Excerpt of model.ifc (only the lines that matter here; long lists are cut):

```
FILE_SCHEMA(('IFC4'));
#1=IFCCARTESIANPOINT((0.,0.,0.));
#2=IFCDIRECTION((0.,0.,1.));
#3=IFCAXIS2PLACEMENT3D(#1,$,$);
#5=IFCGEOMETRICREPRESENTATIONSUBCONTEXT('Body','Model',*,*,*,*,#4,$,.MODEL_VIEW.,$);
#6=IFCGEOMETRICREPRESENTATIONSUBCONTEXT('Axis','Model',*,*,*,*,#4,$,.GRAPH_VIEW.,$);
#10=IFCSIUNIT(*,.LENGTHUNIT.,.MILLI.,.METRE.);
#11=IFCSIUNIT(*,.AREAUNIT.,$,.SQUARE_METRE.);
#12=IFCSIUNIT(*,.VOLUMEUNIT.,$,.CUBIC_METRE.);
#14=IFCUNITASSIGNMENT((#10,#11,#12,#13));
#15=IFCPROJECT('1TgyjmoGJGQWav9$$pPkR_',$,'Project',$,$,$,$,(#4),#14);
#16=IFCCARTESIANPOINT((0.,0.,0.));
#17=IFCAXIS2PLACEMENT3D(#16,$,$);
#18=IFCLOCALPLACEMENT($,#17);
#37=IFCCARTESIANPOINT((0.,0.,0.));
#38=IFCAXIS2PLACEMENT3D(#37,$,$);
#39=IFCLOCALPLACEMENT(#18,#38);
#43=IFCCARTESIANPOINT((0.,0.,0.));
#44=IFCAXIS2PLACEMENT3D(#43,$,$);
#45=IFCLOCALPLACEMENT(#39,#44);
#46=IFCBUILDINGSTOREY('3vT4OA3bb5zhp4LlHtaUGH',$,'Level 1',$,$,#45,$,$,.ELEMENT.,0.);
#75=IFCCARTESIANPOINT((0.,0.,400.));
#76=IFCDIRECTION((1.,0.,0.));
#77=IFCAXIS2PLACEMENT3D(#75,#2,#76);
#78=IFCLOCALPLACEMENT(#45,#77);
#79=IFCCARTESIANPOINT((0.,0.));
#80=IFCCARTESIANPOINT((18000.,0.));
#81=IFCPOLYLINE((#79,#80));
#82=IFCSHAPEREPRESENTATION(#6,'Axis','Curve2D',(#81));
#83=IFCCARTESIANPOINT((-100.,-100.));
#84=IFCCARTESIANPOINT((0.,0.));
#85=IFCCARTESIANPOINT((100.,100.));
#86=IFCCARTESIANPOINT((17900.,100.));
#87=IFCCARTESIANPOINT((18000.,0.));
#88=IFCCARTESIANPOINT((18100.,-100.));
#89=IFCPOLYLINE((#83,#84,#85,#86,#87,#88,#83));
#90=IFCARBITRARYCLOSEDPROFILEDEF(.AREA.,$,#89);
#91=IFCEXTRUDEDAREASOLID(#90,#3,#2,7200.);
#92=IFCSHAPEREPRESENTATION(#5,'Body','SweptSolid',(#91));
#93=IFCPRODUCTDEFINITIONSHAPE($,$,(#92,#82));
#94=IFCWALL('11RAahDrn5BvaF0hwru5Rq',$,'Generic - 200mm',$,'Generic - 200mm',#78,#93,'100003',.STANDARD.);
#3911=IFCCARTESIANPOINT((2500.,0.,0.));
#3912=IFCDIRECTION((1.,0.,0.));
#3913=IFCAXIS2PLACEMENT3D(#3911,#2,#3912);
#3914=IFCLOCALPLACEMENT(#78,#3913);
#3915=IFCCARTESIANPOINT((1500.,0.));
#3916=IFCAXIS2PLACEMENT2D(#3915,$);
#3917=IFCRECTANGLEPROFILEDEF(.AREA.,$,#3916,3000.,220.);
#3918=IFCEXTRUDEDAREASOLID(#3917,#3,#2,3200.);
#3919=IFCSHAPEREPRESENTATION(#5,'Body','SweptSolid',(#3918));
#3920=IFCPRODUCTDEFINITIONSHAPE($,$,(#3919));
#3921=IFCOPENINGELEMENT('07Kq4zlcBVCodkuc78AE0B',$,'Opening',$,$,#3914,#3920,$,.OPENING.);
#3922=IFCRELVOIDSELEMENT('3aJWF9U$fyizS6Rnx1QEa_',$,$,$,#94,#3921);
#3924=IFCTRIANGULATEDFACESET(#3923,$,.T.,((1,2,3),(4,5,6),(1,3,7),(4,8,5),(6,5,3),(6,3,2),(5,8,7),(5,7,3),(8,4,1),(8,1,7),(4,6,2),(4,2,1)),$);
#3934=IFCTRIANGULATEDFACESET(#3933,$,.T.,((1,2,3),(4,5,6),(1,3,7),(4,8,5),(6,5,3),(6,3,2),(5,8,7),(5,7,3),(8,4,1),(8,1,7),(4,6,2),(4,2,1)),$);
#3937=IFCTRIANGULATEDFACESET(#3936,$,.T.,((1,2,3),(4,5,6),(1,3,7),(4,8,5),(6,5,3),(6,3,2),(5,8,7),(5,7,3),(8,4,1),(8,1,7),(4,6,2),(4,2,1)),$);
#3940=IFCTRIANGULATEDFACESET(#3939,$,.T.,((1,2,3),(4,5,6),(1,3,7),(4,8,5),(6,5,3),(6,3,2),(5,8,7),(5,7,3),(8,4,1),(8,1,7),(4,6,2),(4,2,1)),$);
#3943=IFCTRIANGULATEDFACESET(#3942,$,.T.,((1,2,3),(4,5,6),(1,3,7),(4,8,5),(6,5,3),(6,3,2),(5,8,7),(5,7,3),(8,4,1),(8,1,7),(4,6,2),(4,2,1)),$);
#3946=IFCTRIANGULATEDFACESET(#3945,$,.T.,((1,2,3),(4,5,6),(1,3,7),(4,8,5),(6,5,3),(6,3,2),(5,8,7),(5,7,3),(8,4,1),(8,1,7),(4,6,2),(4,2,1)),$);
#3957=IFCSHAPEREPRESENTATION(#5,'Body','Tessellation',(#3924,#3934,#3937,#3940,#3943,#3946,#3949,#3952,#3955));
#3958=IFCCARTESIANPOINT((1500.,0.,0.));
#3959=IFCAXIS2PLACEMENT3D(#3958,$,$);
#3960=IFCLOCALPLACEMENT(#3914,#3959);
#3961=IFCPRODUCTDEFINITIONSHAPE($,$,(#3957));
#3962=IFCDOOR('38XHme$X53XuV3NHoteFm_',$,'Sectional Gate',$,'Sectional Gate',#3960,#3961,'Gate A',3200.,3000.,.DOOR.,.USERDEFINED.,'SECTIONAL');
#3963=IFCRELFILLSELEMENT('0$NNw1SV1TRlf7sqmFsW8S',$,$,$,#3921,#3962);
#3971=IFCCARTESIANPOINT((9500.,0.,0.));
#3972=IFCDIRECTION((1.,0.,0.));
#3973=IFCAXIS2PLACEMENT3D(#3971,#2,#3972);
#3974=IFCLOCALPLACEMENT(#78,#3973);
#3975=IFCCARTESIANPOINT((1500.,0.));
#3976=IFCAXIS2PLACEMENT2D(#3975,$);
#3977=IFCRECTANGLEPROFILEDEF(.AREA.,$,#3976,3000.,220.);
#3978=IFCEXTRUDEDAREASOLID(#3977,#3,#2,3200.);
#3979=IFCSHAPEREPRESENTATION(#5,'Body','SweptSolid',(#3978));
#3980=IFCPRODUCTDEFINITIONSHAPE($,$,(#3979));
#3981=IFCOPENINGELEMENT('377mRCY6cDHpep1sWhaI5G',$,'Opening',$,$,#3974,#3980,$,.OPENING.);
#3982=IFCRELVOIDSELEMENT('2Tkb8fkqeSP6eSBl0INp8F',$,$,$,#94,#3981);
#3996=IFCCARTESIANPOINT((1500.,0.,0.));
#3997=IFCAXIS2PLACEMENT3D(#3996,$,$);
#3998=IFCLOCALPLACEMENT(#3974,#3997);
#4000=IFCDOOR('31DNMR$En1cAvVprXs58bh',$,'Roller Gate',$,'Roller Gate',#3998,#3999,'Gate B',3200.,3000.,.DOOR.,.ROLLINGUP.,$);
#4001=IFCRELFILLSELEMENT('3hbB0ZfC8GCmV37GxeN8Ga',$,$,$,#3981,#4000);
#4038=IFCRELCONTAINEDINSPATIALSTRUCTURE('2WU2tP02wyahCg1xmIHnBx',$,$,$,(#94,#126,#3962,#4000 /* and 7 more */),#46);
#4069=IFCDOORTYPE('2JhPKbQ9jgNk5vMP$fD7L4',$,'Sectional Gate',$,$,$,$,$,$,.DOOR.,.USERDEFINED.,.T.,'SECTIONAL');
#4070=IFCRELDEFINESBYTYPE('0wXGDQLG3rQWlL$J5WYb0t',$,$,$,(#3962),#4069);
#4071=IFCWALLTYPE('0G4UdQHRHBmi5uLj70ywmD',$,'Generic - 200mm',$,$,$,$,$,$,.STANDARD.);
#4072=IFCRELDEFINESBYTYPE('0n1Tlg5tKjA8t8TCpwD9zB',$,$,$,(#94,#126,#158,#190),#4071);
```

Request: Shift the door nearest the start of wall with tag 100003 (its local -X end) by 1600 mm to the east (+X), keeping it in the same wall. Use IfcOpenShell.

```python
import ifcopenshell
import ifcopenshell.api.geometry
import ifcopenshell.util.placement
import ifcopenshell.util.unit

model = ifcopenshell.open("model.ifc")
unit_scale = ifcopenshell.util.unit.calculate_unit_scale(model)

door = model.by_guid("38XHme$X53XuV3NHoteFm_")
opening = door.FillsVoids[0].RelatingOpeningElement
wall = opening.VoidsElements[0].RelatingBuildingElement

wall_matrix = ifcopenshell.util.placement.get_local_placement(wall.ObjectPlacement)
shift = wall_matrix[:3, 0] * 1.6 / unit_scale
before = ifcopenshell.util.placement.get_local_placement(door.ObjectPlacement)[:3, 3].copy()

# The door is placed relative to its opening, so it follows when the opening moves.
matrix = ifcopenshell.util.placement.get_local_placement(opening.ObjectPlacement)
matrix[:3, 3] += shift
ifcopenshell.api.geometry.edit_object_placement(
    model, product=opening, matrix=matrix, is_si=False, should_transform_children=True
)

after = ifcopenshell.util.placement.get_local_placement(door.ObjectPlacement)[:3, 3]
print("door moved by", (after - before).round(3) + 0.0)

model.write("model_rev.ifc")
```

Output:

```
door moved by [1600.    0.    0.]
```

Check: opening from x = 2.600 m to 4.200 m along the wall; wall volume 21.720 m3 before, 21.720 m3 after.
